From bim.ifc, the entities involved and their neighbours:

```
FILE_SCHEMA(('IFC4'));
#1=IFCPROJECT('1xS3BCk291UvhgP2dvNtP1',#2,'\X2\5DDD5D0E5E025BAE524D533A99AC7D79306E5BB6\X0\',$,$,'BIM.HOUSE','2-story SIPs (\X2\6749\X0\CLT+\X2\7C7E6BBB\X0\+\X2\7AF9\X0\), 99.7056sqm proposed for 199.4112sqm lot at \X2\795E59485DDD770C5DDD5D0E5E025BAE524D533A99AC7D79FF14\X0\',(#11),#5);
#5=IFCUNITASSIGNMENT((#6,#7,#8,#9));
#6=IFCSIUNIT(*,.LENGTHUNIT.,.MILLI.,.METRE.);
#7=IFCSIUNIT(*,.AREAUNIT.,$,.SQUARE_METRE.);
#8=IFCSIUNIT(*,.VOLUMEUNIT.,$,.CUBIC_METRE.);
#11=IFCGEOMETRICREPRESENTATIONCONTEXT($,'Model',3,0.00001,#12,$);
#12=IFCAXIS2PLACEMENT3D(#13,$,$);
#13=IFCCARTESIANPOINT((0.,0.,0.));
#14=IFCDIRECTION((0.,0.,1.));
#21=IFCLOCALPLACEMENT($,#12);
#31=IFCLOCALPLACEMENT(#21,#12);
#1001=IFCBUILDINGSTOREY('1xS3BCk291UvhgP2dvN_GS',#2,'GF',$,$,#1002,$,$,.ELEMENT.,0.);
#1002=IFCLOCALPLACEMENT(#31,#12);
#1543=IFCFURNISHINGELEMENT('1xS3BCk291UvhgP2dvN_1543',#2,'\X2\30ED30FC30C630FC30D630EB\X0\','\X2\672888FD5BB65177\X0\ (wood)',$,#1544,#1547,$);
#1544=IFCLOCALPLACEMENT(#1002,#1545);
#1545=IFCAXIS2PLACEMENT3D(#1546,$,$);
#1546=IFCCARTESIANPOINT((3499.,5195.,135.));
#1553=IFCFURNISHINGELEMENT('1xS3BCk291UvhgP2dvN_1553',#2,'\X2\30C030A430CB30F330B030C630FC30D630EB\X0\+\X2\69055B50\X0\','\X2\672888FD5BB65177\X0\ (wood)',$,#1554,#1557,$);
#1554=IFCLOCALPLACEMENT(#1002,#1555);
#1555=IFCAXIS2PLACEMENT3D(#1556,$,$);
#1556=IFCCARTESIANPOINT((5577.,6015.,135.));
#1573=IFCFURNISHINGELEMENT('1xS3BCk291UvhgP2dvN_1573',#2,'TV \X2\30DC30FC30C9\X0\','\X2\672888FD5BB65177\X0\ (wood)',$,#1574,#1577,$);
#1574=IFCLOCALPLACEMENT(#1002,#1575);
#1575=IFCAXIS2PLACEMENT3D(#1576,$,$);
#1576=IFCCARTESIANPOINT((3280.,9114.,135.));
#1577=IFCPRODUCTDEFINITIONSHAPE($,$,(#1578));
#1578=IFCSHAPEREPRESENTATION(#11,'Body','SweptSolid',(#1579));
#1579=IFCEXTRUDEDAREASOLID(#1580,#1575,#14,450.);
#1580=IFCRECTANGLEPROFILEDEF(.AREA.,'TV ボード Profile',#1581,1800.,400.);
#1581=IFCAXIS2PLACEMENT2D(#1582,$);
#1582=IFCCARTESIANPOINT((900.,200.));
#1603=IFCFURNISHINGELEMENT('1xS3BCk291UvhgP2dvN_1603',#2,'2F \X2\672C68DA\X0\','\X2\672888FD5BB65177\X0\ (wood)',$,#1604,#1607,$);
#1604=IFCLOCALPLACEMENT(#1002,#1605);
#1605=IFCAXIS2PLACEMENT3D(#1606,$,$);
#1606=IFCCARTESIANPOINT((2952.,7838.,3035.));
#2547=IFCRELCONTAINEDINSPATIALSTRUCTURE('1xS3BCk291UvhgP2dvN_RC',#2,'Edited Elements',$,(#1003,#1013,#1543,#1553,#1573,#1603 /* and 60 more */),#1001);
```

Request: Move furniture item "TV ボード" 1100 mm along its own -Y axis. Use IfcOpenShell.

```python
import ifcopenshell
import ifcopenshell.api.geometry
import ifcopenshell.util.placement

model = ifcopenshell.open("bim.ifc")

item = model.by_id(1573)
matrix = ifcopenshell.util.placement.get_local_placement(item.ObjectPlacement)
matrix[:3, 3] -= matrix[:3, 1] * 1100.0
ifcopenshell.api.geometry.edit_object_placement(model, product=item, matrix=matrix, is_si=False)

print(ifcopenshell.util.placement.get_local_placement(item.ObjectPlacement).round(3) + 0.0)

model.write("bim_edited.ifc")
```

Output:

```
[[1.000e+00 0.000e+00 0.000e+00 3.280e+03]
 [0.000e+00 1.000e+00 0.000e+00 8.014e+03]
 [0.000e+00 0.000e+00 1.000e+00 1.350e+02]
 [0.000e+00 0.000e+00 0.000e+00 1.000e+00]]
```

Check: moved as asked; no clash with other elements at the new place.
